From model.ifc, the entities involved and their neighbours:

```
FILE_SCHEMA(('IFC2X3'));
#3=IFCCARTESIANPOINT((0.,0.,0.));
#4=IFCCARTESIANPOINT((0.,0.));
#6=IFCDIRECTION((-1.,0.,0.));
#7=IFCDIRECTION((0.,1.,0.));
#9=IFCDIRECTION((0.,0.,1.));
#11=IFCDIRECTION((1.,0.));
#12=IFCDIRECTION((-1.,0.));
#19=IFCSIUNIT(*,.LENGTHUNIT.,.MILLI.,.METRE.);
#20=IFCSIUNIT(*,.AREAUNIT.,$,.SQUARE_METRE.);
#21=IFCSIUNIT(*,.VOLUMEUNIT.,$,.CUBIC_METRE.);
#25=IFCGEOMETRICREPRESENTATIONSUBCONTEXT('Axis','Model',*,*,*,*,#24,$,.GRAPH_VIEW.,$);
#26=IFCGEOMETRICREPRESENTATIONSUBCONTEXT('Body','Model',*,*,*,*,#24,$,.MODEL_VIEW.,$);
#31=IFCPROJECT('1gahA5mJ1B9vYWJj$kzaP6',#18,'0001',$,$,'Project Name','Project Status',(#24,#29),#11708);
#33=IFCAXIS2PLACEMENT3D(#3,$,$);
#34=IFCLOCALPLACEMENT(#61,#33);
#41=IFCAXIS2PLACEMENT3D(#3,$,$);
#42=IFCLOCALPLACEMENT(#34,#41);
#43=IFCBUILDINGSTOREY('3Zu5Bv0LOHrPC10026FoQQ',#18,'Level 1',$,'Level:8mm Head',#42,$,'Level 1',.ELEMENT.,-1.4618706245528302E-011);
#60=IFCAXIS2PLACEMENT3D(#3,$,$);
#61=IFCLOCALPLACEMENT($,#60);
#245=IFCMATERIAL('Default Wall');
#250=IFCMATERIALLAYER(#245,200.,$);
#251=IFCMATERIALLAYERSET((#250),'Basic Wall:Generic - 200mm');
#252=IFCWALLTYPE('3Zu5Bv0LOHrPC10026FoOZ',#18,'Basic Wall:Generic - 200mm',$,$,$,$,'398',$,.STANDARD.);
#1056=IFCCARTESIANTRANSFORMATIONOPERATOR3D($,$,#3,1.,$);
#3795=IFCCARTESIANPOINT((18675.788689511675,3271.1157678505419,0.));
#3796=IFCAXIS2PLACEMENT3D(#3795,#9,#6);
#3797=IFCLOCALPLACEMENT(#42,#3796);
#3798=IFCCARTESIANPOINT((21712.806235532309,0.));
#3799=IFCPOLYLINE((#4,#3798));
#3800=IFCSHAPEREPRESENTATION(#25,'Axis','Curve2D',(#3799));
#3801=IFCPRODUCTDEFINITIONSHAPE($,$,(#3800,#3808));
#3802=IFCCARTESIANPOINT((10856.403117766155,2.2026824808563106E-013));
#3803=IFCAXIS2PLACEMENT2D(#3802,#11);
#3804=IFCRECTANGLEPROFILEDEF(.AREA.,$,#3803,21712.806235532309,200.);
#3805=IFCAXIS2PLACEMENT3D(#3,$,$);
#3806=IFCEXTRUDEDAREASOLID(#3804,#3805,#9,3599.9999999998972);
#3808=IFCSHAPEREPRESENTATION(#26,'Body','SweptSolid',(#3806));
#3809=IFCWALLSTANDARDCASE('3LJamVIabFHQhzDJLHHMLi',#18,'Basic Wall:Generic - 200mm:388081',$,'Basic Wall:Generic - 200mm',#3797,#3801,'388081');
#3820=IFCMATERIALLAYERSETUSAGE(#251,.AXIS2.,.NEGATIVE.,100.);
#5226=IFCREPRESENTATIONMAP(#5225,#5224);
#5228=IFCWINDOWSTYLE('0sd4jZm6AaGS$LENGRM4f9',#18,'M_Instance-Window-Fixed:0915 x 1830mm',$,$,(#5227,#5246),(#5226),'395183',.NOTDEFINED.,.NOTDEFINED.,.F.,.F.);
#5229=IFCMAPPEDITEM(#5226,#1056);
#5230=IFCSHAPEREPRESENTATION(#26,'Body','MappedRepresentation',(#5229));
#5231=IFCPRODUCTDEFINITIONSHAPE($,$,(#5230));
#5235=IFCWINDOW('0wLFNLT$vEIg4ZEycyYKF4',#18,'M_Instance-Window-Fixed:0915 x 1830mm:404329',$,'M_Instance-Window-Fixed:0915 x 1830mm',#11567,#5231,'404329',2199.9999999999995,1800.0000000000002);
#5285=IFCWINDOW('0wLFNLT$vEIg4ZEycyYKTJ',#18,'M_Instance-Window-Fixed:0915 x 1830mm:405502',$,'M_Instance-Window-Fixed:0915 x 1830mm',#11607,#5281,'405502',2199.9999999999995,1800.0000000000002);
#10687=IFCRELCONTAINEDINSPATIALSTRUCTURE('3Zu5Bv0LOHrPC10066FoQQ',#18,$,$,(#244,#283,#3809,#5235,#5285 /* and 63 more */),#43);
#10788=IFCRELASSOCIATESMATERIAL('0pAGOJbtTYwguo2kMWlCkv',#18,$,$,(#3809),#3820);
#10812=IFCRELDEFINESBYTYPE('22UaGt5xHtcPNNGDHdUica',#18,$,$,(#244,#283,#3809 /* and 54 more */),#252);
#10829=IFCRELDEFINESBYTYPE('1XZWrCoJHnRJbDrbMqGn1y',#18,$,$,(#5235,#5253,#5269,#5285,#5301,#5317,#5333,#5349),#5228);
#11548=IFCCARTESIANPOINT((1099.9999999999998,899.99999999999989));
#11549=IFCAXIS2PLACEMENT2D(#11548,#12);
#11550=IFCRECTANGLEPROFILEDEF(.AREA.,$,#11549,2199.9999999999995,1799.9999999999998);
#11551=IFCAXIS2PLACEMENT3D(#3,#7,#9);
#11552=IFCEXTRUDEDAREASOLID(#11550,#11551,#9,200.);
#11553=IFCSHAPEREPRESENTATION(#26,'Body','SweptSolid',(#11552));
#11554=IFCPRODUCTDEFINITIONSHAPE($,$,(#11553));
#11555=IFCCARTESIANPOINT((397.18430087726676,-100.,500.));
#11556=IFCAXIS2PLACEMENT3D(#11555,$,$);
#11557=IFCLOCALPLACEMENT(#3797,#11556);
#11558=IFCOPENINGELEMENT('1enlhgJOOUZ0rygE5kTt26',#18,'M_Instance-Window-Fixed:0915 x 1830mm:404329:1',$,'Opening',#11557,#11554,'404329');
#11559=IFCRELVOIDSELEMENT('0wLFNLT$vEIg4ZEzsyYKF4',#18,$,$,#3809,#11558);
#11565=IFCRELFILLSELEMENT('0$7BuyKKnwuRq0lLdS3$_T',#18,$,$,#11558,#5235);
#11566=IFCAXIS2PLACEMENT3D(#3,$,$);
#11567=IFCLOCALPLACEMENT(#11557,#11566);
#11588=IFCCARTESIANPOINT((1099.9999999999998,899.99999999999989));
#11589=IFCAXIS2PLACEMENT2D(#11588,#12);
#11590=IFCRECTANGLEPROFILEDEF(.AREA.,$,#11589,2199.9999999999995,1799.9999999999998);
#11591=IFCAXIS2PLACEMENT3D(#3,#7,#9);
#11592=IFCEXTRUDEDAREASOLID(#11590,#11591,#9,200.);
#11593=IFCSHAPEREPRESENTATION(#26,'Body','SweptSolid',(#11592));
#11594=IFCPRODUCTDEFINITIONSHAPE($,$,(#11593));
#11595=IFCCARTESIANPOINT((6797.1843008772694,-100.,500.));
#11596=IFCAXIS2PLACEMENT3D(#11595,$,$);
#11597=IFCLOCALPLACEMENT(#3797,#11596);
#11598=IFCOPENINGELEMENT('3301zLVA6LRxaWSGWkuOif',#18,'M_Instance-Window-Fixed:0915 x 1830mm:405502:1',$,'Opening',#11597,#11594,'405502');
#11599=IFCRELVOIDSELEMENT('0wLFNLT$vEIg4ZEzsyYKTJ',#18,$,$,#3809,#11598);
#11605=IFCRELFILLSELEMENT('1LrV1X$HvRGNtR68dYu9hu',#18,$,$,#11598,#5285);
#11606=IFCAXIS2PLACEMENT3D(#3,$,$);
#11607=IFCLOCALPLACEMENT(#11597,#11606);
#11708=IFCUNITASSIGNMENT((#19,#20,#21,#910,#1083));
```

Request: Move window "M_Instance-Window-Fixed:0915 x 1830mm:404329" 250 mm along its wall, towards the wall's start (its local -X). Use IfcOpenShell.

```python
import ifcopenshell
import ifcopenshell.api.geometry
import ifcopenshell.util.placement
import ifcopenshell.util.unit

model = ifcopenshell.open("model.ifc")
unit_scale = ifcopenshell.util.unit.calculate_unit_scale(model)

window = model.by_id(5235)
opening = window.FillsVoids[0].RelatingOpeningElement
wall = opening.VoidsElements[0].RelatingBuildingElement

wall_matrix = ifcopenshell.util.placement.get_local_placement(wall.ObjectPlacement)
shift = wall_matrix[:3, 0] * -0.25 / unit_scale
before = ifcopenshell.util.placement.get_local_placement(window.ObjectPlacement)[:3, 3].copy()

# The window is placed relative to its opening, so it follows when the opening moves.
matrix = ifcopenshell.util.placement.get_local_placement(opening.ObjectPlacement)
matrix[:3, 3] += shift
ifcopenshell.api.geometry.edit_object_placement(
    model, product=opening, matrix=matrix, is_si=False, should_transform_children=True
)

after = ifcopenshell.util.placement.get_local_placement(window.ObjectPlacement)[:3, 3]
print("window moved by", (after - before).round(3) + 0.0)

model.write("model-out.ifc")
```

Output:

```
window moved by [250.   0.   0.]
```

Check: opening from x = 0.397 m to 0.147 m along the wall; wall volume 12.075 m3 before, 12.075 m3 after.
